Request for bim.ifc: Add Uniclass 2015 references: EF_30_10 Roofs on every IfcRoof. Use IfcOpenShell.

First a look at what the model holds.

```python
import ifcopenshell

model = ifcopenshell.open("bim.ifc")
print(model.schema)
print("classifications:", [c.Name for c in model.by_type("IfcClassification")])
for ifc_class in ("IfcDoor", "IfcRoof", "IfcStair", "IfcWall", "IfcWindow"):
    print(ifc_class, len(model.by_type(ifc_class)))
```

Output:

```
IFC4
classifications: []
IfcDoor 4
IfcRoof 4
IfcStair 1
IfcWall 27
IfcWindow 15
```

```python
import ifcopenshell
import ifcopenshell.api.classification

model = ifcopenshell.open("bim.ifc")

system = ifcopenshell.api.classification.add_classification(model, classification="Uniclass 2015")

codes = {
    "IfcRoof": ("EF_30_10", "Roofs"),
}
for ifc_class, (code, name) in codes.items():
    products = model.by_type(ifc_class)
    ifcopenshell.api.classification.add_reference(
        model, products=products, classification=system, identification=code, name=name
    )
    print(code, len(products))

model.write("bim-out.ifc")
```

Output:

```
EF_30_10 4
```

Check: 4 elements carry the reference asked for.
